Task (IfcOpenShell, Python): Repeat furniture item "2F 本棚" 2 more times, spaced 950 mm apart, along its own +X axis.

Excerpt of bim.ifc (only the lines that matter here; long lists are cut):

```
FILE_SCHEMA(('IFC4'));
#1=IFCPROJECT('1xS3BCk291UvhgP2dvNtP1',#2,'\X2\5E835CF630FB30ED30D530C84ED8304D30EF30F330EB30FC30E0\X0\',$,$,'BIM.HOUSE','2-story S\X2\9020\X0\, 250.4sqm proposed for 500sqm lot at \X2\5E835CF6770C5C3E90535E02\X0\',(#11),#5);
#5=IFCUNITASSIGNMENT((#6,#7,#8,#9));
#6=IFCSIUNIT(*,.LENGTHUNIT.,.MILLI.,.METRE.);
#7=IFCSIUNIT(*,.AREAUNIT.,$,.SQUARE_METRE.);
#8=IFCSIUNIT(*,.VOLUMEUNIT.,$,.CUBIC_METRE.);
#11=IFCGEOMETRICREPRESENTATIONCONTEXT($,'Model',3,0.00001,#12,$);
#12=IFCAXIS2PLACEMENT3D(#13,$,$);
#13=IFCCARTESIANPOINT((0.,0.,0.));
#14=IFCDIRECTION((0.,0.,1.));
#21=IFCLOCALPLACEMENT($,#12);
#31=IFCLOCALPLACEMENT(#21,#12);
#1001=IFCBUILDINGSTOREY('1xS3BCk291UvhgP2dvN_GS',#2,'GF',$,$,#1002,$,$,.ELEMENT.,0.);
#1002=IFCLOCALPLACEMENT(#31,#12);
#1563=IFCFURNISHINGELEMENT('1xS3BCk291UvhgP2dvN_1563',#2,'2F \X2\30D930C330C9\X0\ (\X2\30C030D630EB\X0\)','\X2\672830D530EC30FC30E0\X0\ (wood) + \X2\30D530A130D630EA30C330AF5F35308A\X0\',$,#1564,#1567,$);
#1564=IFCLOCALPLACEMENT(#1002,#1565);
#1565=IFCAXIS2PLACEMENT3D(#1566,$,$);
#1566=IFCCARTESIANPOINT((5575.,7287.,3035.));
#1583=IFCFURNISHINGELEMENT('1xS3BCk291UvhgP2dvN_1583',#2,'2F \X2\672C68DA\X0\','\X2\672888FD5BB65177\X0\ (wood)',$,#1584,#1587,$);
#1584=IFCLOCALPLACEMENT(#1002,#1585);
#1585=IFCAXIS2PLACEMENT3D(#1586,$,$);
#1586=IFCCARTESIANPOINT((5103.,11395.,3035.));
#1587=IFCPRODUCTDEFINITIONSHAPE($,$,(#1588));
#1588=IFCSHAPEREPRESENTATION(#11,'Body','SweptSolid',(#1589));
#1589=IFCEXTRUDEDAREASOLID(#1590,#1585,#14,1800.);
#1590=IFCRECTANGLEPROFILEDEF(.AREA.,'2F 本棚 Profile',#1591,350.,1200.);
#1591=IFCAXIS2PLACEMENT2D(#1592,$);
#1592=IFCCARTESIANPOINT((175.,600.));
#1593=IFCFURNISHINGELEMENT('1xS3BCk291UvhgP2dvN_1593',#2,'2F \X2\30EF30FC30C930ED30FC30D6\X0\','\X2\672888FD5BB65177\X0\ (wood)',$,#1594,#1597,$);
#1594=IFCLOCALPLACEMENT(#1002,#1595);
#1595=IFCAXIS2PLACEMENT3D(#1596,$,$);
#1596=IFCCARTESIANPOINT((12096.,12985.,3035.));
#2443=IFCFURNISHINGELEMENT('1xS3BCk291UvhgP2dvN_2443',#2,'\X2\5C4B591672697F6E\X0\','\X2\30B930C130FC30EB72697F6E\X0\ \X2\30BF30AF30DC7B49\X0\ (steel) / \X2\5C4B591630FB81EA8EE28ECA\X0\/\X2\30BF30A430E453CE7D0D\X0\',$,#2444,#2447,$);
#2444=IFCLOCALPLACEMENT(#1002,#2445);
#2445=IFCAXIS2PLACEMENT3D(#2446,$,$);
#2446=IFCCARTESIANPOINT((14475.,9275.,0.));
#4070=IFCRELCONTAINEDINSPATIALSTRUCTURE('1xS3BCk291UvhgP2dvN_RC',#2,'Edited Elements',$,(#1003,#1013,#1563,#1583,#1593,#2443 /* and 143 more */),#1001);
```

```python
import ifcopenshell
import ifcopenshell.api.geometry
import ifcopenshell.api.root
import ifcopenshell.util.element
import ifcopenshell.util.placement
import ifcopenshell.util.unit

model = ifcopenshell.open("bim.ifc")
unit_scale = ifcopenshell.util.unit.calculate_unit_scale(model)


def reuse_history(source, copy):
    """copy_class also copies each property set's owner history, people and application; keep the originals."""
    for rel in copy.IsDefinedBy:
        if rel.is_a("IfcRelDefinesByProperties") and (history := rel.RelatingPropertyDefinition.OwnerHistory):
            rel.RelatingPropertyDefinition.OwnerHistory = source.OwnerHistory
            ifcopenshell.util.element.remove_deep2(model, history)


source = model.by_guid("1xS3BCk291UvhgP2dvN_1583")
base = ifcopenshell.util.placement.get_local_placement(source.ObjectPlacement)
step = base[:3, 0] * 0.95 / unit_scale

for i in range(1, 3):
    copy = ifcopenshell.api.root.copy_class(model, product=source)
    copy.Representation = ifcopenshell.util.element.copy_deep(
        model, source.Representation, exclude=["IfcGeometricRepresentationContext", "IfcRepresentationMap"]
    )
    reuse_history(source, copy)
    matrix = base.copy()
    matrix[:3, 3] += i * step
    print("added at", matrix[:3, 3].round(3) + 0.0)
    ifcopenshell.api.geometry.edit_object_placement(model, product=copy, matrix=matrix, is_si=False)

model.write("bim_rev.ifc")
```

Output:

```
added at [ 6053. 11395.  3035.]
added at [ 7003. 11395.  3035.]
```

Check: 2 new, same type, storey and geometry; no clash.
